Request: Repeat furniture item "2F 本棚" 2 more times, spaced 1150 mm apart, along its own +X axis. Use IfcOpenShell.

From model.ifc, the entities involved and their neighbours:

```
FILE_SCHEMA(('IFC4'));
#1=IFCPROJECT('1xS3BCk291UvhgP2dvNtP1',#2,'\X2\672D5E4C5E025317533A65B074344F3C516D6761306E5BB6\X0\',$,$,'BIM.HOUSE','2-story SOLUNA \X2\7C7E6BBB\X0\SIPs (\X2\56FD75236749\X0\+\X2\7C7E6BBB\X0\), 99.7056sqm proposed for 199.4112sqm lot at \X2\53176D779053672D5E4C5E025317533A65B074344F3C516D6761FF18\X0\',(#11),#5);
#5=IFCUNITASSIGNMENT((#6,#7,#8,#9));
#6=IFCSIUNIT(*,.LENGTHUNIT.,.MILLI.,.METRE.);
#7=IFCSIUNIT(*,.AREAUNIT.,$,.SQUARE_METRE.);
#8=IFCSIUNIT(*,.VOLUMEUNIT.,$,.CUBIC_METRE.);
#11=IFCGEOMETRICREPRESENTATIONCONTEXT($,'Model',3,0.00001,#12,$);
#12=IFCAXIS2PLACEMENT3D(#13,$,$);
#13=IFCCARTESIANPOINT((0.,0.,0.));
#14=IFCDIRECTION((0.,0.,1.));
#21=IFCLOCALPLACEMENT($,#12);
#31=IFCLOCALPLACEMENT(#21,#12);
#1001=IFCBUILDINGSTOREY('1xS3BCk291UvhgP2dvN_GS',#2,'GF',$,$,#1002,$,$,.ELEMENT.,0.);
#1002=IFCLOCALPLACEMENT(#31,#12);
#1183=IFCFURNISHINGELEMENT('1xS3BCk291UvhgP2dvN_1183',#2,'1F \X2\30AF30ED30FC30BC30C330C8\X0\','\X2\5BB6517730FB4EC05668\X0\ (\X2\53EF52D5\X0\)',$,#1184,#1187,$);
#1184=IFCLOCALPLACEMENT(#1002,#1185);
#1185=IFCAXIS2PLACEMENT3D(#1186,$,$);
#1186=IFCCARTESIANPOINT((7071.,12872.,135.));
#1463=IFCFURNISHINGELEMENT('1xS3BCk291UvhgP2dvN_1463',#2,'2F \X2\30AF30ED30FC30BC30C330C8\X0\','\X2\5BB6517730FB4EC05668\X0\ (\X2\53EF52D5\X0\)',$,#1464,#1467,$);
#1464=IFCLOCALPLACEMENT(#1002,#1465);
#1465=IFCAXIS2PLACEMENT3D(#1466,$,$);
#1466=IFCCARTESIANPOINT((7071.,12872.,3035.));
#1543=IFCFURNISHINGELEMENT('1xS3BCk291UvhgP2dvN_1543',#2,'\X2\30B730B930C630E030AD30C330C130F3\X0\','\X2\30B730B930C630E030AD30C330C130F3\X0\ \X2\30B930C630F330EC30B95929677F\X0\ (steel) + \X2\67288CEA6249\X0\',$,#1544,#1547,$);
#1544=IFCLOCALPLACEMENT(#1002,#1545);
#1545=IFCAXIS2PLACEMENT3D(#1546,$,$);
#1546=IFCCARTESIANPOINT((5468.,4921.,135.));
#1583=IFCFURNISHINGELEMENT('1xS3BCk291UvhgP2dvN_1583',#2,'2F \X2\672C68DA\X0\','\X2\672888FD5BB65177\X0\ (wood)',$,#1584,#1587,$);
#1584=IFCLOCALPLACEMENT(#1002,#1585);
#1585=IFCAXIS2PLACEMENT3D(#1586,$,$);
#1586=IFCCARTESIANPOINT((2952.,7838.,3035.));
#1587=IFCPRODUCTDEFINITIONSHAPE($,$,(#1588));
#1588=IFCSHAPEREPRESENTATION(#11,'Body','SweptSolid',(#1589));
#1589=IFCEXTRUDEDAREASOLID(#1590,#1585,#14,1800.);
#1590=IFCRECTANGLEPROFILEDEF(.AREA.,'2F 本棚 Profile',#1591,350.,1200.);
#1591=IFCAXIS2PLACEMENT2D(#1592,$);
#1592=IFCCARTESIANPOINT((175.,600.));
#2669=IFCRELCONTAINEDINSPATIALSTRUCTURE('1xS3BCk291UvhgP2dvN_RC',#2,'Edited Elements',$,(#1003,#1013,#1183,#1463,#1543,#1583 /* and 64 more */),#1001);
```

```python
import ifcopenshell
import ifcopenshell.api.geometry
import ifcopenshell.api.root
import ifcopenshell.util.element
import ifcopenshell.util.placement

model = ifcopenshell.open("model.ifc")


def reuse_history(source, copy):
    """copy_class also copies each property set's owner history, people and application; keep the originals."""
    for rel in copy.IsDefinedBy:
        if rel.is_a("IfcRelDefinesByProperties") and (history := rel.RelatingPropertyDefinition.OwnerHistory):
            rel.RelatingPropertyDefinition.OwnerHistory = source.OwnerHistory
            ifcopenshell.util.element.remove_deep2(model, history)


source = model.by_id(1583)
base = ifcopenshell.util.placement.get_local_placement(source.ObjectPlacement)
step = base[:3, 0] * 1150.0

for i in range(1, 3):
    copy = ifcopenshell.api.root.copy_class(model, product=source)
    copy.Representation = ifcopenshell.util.element.copy_deep(
        model, source.Representation, exclude=["IfcGeometricRepresentationContext", "IfcRepresentationMap"]
    )
    reuse_history(source, copy)
    matrix = base.copy()
    matrix[:3, 3] += i * step
    print("added at", matrix[:3, 3].round(3) + 0.0)
    ifcopenshell.api.geometry.edit_object_placement(model, product=copy, matrix=matrix, is_si=False)

model.write("model_edited.ifc")
```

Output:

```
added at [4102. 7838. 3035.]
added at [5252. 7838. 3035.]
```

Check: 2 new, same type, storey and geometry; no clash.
